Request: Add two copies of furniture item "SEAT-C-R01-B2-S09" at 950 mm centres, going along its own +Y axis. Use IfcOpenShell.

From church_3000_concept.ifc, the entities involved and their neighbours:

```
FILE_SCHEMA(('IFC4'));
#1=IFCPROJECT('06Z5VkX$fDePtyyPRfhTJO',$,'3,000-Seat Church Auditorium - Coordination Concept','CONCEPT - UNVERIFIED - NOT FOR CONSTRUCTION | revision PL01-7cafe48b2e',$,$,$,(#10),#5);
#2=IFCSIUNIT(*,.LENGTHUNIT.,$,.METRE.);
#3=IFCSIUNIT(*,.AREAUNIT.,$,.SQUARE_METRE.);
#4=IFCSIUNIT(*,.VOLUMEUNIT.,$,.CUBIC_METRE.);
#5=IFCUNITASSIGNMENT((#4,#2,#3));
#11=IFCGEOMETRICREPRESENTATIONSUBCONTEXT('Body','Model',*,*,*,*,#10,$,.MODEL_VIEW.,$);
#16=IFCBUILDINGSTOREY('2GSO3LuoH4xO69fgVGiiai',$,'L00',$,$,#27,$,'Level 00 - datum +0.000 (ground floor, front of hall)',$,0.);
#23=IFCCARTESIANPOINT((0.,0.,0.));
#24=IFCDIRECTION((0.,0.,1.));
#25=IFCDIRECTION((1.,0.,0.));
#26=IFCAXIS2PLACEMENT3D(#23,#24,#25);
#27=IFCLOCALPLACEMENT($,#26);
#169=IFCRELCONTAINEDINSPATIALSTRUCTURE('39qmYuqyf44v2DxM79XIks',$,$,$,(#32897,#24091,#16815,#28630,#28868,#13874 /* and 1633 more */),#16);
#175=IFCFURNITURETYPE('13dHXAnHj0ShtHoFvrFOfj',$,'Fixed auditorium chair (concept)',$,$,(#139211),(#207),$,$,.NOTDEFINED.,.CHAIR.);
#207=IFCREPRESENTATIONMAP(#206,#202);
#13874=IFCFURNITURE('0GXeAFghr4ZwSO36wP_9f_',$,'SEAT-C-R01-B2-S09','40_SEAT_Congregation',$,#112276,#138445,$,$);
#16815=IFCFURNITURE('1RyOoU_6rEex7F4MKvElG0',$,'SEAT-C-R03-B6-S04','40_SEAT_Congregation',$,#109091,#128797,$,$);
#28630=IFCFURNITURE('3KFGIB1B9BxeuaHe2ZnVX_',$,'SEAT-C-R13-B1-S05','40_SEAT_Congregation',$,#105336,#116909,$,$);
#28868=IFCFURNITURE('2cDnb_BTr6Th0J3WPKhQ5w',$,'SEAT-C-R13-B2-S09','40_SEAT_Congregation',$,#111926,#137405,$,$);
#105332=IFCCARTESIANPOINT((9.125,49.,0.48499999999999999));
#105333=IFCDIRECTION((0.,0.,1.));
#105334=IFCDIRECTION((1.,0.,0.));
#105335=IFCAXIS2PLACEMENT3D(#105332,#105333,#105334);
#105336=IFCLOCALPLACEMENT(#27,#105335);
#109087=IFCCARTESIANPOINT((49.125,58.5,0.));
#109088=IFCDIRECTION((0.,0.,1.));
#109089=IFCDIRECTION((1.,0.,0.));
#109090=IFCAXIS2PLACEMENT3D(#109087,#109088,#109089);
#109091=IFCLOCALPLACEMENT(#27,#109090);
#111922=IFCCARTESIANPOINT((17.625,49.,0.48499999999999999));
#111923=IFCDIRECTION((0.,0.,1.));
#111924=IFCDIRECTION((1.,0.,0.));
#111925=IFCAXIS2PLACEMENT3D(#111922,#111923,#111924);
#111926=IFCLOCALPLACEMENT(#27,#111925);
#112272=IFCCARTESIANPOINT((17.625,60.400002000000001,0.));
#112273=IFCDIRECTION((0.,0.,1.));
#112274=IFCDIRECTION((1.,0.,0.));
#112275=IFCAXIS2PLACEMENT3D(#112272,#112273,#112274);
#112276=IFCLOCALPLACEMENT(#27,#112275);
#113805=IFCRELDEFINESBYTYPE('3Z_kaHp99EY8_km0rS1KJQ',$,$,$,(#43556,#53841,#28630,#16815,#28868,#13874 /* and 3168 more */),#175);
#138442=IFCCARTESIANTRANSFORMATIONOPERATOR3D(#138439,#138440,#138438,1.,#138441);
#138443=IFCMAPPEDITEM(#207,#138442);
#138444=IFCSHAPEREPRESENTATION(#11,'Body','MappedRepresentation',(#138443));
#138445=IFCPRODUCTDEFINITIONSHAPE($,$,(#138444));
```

```python
import ifcopenshell
import ifcopenshell.api.geometry
import ifcopenshell.api.root
import ifcopenshell.util.element
import ifcopenshell.util.placement
import ifcopenshell.util.unit

model = ifcopenshell.open("church_3000_concept.ifc")
unit_scale = ifcopenshell.util.unit.calculate_unit_scale(model)

source = model.by_guid("0GXeAFghr4ZwSO36wP_9f_")
base = ifcopenshell.util.placement.get_local_placement(source.ObjectPlacement)
step = base[:3, 1] * 0.95 / unit_scale

for i in range(1, 3):
    copy = ifcopenshell.api.root.copy_class(model, product=source)
    copy.Representation = ifcopenshell.util.element.copy_deep(
        model, source.Representation, exclude=["IfcGeometricRepresentationContext", "IfcRepresentationMap"]
    )
    matrix = base.copy()
    matrix[:3, 3] += i * step
    print("added at", matrix[:3, 3].round(3) + 0.0)
    ifcopenshell.api.geometry.edit_object_placement(model, product=copy, matrix=matrix, is_si=False)

model.write("church_3000_concept_edited.ifc")
```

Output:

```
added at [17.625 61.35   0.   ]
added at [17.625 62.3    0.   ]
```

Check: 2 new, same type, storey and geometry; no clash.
